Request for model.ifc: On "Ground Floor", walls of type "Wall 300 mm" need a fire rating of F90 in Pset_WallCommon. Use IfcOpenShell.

First a look at what the model holds.

```python
import ifcopenshell
import ifcopenshell.util.element

model = ifcopenshell.open("model.ifc")
print(model.schema)
storey = next(s for s in model.by_type("IfcBuildingStorey") if s.Name == "Ground Floor")
walls = [e for e in ifcopenshell.util.element.get_decomposition(storey) if e.is_a("IfcWall")]
seen = {}
for e in walls:
    element_type = ifcopenshell.util.element.get_type(e)
    key = (element_type.Name if element_type != e and element_type else None, ifcopenshell.util.element.get_pset(e, "Pset_WallCommon", "FireRating"))
    seen[key] = seen.get(key, 0) + 1
for (name, value), count in sorted(seen.items(), key=str):
    print(count, "x", name, "|", value)
```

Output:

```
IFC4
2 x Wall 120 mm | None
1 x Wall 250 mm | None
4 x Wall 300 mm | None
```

```python
import ifcopenshell
import ifcopenshell.api.pset
import ifcopenshell.util.element

model = ifcopenshell.open("model.ifc")

storey = next(s for s in model.by_type("IfcBuildingStorey") if s.Name == "Ground Floor")
walls = [e for e in ifcopenshell.util.element.get_decomposition(storey) if e.is_a("IfcWall")]

count = 0
for e in walls:
    element_type = ifcopenshell.util.element.get_type(e)
    if element_type in (None, e) or element_type.Name != "Wall 300 mm":
        continue
    # add_pset returns the element's existing set when there is one.
    pset = ifcopenshell.api.pset.add_pset(model, product=e, name="Pset_WallCommon")
    ifcopenshell.api.pset.edit_pset(model, pset=pset, properties={"FireRating": "F90"})
    count += 1

print(count, "walls updated")

model.write("model-out.ifc")
```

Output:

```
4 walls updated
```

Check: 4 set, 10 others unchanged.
